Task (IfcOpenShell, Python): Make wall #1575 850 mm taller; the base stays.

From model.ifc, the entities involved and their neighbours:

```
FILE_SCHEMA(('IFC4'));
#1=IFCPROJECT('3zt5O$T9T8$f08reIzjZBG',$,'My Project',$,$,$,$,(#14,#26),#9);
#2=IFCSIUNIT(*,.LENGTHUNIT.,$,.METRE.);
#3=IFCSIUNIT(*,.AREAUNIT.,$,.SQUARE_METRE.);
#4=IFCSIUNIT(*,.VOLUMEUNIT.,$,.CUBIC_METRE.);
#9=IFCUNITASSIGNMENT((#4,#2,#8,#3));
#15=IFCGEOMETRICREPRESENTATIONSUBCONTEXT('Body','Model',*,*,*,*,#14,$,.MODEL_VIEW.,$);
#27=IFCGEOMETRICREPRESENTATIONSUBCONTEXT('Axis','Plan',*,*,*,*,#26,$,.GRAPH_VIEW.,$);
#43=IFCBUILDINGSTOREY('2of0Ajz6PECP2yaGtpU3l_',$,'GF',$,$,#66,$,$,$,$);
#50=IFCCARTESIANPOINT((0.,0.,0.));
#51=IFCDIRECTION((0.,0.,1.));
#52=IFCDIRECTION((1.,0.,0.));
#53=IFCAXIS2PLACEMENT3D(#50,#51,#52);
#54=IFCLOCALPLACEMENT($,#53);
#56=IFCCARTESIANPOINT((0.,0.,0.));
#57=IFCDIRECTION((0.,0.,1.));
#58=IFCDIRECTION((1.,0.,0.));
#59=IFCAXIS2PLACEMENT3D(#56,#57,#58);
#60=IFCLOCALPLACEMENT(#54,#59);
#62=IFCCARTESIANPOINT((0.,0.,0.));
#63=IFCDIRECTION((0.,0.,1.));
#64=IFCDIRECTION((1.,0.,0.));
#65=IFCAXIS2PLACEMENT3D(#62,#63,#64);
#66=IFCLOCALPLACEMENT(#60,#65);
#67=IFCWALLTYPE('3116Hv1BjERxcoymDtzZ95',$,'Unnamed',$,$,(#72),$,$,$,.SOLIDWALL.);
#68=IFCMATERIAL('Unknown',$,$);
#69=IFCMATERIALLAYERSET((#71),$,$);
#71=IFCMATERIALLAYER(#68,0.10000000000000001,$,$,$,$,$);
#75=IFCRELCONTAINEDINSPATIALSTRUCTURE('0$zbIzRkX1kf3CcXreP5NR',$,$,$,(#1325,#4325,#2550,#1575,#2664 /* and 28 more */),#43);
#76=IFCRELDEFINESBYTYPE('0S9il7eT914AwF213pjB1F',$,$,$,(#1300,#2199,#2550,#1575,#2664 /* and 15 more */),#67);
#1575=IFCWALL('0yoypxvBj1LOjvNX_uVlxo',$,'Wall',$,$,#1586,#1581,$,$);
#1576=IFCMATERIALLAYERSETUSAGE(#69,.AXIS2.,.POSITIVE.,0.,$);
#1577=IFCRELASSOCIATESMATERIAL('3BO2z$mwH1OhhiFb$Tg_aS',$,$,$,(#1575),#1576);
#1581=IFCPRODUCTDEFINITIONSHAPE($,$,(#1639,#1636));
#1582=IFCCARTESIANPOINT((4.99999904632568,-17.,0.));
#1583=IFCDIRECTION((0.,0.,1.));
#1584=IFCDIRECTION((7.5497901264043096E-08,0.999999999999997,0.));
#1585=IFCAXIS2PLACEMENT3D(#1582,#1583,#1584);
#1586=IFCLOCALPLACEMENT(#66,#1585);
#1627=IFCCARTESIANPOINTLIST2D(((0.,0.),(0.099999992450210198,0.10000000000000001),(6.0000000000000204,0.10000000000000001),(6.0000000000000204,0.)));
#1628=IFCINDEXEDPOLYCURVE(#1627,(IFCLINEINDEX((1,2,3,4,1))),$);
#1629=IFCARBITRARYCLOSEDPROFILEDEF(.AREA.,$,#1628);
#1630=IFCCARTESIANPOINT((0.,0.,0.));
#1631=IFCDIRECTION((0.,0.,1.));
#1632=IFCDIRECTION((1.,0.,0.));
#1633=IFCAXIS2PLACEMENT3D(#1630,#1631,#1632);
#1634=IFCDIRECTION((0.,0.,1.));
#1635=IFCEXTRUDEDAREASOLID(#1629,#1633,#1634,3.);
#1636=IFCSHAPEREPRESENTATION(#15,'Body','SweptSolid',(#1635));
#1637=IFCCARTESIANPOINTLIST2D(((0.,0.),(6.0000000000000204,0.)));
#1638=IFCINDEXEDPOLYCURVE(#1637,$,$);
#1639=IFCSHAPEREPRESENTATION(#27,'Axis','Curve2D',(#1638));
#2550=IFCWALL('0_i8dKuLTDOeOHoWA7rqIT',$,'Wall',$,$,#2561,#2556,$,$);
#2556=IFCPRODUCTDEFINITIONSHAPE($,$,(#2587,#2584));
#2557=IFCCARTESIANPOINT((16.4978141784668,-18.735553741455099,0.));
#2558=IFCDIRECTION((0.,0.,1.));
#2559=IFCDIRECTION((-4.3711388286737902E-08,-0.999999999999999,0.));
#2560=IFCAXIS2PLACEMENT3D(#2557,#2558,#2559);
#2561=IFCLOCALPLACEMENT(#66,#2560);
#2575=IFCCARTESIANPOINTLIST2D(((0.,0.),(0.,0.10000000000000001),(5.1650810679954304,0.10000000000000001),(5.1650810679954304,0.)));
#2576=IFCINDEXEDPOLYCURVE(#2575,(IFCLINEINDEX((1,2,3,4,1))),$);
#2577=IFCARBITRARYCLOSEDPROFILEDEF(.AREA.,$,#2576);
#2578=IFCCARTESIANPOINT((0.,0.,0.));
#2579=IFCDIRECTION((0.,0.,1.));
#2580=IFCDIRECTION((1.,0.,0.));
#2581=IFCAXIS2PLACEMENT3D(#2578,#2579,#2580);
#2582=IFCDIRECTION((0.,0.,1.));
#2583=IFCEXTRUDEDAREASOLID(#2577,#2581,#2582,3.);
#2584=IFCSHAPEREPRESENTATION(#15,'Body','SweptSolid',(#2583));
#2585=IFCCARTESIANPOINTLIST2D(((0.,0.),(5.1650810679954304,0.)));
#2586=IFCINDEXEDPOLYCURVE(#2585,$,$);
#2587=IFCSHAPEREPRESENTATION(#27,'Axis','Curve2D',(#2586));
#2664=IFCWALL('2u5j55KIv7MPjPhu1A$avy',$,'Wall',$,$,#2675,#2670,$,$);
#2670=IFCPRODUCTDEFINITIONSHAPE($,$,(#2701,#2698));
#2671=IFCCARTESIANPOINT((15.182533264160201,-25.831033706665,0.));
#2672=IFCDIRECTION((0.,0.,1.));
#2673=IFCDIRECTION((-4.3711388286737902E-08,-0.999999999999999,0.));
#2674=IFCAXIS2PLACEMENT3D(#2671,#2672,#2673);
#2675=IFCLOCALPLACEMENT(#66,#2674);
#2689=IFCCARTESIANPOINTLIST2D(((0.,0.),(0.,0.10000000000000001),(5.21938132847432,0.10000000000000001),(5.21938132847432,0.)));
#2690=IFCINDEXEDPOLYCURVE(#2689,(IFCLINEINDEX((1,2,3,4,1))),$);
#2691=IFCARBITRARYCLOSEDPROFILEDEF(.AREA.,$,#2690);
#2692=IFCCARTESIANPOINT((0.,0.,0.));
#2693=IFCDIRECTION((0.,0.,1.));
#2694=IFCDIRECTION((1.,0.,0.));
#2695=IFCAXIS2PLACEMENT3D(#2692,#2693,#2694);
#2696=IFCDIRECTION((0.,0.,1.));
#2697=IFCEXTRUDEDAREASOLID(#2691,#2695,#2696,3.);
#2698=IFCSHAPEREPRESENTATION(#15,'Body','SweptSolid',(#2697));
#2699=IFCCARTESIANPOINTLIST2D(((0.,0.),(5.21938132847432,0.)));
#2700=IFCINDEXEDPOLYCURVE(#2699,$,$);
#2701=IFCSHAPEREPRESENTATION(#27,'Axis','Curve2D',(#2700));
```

```python
import ifcopenshell
import ifcopenshell.geom
import ifcopenshell.util.representation
import ifcopenshell.util.shape

model = ifcopenshell.open("model.ifc")
settings = ifcopenshell.geom.settings()


def volume(element):
    """Net volume in cubic metres, openings subtracted."""
    shape = ifcopenshell.geom.create_shape(settings, element)
    return ifcopenshell.util.shape.get_volume(shape.geometry)


wall = model.by_guid("0yoypxvBj1LOjvNX_uVlxo")
before = volume(wall)

body = ifcopenshell.util.representation.get_representation(wall, "Model", "Body")
solid = body.Items[0]
old_height = solid.Depth
solid.Depth += 0.85
after = volume(wall)

print(f"height {old_height:g} -> {solid.Depth:g}, volume {before:.3f} -> {after:.3f} m3")

model.write("model_updated.ifc")
```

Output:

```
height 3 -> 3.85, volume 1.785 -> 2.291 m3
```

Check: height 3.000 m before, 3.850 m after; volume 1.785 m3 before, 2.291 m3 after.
